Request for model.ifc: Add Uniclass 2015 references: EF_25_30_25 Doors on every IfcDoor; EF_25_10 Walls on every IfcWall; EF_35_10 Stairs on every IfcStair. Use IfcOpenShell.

First a look at what the model holds.

```python
import ifcopenshell

model = ifcopenshell.open("model.ifc")
print(model.schema)
print("classifications:", [c.Name for c in model.by_type("IfcClassification")])
for ifc_class in ("IfcDoor", "IfcRoof", "IfcStair", "IfcWall", "IfcWindow"):
    print(ifc_class, len(model.by_type(ifc_class)))
```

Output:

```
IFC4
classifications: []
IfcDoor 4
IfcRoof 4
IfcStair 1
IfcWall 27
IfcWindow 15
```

```python
import ifcopenshell
import ifcopenshell.api.classification

model = ifcopenshell.open("model.ifc")

system = ifcopenshell.api.classification.add_classification(model, classification="Uniclass 2015")

codes = {
    "IfcDoor": ("EF_25_30_25", "Doors"),
    "IfcWall": ("EF_25_10", "Walls"),
    "IfcStair": ("EF_35_10", "Stairs"),
}
for ifc_class, (code, name) in codes.items():
    products = model.by_type(ifc_class)
    ifcopenshell.api.classification.add_reference(
        model, products=products, classification=system, identification=code, name=name
    )
    print(code, len(products))

model.write("model_updated.ifc")
```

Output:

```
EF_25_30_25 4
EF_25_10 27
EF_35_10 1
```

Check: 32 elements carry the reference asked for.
